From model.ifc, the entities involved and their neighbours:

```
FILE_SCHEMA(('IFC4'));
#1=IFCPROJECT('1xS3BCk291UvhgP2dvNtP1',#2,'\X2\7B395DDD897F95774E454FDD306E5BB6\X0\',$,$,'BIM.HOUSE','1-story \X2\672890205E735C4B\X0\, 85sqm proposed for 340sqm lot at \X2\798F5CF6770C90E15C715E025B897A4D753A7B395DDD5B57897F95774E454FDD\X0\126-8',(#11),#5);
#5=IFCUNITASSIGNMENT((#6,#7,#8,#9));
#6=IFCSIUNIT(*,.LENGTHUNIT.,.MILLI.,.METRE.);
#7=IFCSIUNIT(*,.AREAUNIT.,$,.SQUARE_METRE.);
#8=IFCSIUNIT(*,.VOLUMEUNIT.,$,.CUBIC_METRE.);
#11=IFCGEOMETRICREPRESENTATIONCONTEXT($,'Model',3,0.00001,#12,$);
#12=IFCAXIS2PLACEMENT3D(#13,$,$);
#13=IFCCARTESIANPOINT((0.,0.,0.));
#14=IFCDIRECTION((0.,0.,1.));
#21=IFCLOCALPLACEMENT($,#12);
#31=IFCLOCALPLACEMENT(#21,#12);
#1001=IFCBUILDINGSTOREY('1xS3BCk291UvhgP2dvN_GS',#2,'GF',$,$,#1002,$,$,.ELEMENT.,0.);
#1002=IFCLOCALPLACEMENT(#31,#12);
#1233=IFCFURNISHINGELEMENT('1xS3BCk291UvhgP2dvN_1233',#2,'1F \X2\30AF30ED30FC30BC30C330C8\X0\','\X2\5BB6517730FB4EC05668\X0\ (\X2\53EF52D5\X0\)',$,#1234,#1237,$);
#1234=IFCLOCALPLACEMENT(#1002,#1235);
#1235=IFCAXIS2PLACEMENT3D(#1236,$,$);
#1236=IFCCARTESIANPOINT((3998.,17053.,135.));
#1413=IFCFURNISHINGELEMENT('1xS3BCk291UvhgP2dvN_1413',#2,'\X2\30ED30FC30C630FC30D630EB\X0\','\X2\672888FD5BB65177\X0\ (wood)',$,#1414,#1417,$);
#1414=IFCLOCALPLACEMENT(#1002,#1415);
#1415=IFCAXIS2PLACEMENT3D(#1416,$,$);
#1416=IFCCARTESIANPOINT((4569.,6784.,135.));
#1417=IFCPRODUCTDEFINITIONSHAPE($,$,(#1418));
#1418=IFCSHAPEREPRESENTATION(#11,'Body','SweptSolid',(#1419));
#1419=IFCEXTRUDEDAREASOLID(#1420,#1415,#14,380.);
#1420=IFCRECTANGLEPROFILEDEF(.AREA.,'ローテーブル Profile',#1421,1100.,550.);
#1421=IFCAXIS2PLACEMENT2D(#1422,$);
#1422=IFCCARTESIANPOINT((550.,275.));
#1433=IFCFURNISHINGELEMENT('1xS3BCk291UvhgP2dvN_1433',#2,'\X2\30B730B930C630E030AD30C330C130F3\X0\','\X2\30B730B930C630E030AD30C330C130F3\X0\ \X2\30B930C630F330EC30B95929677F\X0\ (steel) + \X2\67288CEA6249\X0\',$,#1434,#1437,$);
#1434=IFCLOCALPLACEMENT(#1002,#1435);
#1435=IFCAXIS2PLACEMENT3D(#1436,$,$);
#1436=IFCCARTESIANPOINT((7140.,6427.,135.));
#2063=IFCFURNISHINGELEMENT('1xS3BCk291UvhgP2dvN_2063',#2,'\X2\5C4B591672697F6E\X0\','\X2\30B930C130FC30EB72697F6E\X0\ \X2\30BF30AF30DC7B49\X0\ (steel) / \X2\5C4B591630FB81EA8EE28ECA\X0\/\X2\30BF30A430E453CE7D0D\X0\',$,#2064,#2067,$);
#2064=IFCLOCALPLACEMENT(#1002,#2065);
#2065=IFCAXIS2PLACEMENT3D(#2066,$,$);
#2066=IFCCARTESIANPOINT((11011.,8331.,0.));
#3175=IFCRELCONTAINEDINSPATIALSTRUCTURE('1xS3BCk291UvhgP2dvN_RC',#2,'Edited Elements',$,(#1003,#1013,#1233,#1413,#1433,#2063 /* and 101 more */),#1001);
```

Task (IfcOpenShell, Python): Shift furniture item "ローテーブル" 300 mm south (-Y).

```python
import ifcopenshell
import ifcopenshell.api.geometry
import ifcopenshell.util.placement

model = ifcopenshell.open("model.ifc")

item = model.by_guid("1xS3BCk291UvhgP2dvN_1413")
matrix = ifcopenshell.util.placement.get_local_placement(item.ObjectPlacement)
matrix[1, 3] -= 300.0
ifcopenshell.api.geometry.edit_object_placement(model, product=item, matrix=matrix, is_si=False)

print(ifcopenshell.util.placement.get_local_placement(item.ObjectPlacement).round(3) + 0.0)

model.write("model_v2.ifc")
```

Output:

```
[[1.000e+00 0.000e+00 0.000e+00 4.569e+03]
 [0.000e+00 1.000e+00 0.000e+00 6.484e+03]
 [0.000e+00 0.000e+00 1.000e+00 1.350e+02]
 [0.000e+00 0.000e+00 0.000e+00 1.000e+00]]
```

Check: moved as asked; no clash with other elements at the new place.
